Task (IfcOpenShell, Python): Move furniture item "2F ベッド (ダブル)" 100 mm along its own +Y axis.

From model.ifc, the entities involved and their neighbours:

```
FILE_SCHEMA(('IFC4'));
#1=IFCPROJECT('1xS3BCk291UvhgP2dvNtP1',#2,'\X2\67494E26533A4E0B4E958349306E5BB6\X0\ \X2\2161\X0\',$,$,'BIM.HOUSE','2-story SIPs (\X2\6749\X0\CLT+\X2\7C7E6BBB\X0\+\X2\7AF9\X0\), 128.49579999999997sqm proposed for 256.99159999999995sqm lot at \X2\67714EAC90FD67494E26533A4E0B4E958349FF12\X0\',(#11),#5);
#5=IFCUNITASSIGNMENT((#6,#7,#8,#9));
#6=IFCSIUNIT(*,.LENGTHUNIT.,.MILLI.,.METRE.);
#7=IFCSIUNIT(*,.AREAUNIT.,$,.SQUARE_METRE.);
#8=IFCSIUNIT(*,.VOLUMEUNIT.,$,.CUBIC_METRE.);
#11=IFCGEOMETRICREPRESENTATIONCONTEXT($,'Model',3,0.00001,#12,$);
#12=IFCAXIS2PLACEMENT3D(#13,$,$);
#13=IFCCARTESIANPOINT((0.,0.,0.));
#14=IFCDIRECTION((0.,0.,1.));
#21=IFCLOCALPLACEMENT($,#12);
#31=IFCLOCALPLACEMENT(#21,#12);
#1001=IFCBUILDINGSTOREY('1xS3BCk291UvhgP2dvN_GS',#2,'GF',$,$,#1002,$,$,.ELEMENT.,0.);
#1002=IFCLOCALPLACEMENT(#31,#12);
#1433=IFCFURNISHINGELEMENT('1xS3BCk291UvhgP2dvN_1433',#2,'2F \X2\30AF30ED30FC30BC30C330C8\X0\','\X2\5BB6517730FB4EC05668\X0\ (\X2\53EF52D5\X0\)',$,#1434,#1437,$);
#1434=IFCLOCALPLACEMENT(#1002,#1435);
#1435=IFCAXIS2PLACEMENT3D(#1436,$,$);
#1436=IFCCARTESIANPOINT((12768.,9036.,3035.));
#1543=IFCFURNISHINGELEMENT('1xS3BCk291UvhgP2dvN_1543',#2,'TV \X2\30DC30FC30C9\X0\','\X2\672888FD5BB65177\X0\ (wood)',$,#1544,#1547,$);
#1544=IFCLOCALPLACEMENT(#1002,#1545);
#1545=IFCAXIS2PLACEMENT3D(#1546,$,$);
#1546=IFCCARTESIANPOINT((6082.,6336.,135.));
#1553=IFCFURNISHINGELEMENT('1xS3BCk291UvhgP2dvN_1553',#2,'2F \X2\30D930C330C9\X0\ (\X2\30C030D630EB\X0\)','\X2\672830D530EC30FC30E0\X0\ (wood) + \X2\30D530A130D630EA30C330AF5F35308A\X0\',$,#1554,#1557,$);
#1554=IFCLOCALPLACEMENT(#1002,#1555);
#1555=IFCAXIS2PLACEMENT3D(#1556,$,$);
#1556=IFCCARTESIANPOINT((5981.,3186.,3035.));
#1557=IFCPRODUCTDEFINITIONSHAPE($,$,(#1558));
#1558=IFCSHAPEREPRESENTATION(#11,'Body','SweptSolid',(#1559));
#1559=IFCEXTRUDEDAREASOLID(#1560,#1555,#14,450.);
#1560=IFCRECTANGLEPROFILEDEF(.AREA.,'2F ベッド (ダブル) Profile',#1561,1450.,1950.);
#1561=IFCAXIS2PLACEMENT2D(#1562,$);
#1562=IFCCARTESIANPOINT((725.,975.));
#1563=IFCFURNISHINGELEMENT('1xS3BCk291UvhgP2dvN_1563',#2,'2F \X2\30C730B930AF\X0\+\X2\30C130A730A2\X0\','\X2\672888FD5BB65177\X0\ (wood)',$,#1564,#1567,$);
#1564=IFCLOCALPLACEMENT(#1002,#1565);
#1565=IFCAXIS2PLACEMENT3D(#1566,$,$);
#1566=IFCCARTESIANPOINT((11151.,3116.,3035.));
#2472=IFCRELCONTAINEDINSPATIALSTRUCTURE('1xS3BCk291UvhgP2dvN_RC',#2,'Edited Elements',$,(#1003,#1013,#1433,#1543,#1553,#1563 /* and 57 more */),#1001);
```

```python
import ifcopenshell
import ifcopenshell.api.geometry
import ifcopenshell.util.placement
import ifcopenshell.util.unit

model = ifcopenshell.open("model.ifc")
unit_scale = ifcopenshell.util.unit.calculate_unit_scale(model)

item = model.by_guid("1xS3BCk291UvhgP2dvN_1553")
matrix = ifcopenshell.util.placement.get_local_placement(item.ObjectPlacement)
matrix[:3, 3] += matrix[:3, 1] * 0.1 / unit_scale
ifcopenshell.api.geometry.edit_object_placement(model, product=item, matrix=matrix, is_si=False)

print(ifcopenshell.util.placement.get_local_placement(item.ObjectPlacement).round(3) + 0.0)

model.write("model-out.ifc")
```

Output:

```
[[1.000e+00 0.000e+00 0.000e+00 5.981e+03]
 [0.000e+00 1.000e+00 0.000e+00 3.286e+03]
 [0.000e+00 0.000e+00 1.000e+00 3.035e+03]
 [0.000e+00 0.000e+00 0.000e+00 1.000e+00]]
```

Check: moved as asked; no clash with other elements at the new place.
